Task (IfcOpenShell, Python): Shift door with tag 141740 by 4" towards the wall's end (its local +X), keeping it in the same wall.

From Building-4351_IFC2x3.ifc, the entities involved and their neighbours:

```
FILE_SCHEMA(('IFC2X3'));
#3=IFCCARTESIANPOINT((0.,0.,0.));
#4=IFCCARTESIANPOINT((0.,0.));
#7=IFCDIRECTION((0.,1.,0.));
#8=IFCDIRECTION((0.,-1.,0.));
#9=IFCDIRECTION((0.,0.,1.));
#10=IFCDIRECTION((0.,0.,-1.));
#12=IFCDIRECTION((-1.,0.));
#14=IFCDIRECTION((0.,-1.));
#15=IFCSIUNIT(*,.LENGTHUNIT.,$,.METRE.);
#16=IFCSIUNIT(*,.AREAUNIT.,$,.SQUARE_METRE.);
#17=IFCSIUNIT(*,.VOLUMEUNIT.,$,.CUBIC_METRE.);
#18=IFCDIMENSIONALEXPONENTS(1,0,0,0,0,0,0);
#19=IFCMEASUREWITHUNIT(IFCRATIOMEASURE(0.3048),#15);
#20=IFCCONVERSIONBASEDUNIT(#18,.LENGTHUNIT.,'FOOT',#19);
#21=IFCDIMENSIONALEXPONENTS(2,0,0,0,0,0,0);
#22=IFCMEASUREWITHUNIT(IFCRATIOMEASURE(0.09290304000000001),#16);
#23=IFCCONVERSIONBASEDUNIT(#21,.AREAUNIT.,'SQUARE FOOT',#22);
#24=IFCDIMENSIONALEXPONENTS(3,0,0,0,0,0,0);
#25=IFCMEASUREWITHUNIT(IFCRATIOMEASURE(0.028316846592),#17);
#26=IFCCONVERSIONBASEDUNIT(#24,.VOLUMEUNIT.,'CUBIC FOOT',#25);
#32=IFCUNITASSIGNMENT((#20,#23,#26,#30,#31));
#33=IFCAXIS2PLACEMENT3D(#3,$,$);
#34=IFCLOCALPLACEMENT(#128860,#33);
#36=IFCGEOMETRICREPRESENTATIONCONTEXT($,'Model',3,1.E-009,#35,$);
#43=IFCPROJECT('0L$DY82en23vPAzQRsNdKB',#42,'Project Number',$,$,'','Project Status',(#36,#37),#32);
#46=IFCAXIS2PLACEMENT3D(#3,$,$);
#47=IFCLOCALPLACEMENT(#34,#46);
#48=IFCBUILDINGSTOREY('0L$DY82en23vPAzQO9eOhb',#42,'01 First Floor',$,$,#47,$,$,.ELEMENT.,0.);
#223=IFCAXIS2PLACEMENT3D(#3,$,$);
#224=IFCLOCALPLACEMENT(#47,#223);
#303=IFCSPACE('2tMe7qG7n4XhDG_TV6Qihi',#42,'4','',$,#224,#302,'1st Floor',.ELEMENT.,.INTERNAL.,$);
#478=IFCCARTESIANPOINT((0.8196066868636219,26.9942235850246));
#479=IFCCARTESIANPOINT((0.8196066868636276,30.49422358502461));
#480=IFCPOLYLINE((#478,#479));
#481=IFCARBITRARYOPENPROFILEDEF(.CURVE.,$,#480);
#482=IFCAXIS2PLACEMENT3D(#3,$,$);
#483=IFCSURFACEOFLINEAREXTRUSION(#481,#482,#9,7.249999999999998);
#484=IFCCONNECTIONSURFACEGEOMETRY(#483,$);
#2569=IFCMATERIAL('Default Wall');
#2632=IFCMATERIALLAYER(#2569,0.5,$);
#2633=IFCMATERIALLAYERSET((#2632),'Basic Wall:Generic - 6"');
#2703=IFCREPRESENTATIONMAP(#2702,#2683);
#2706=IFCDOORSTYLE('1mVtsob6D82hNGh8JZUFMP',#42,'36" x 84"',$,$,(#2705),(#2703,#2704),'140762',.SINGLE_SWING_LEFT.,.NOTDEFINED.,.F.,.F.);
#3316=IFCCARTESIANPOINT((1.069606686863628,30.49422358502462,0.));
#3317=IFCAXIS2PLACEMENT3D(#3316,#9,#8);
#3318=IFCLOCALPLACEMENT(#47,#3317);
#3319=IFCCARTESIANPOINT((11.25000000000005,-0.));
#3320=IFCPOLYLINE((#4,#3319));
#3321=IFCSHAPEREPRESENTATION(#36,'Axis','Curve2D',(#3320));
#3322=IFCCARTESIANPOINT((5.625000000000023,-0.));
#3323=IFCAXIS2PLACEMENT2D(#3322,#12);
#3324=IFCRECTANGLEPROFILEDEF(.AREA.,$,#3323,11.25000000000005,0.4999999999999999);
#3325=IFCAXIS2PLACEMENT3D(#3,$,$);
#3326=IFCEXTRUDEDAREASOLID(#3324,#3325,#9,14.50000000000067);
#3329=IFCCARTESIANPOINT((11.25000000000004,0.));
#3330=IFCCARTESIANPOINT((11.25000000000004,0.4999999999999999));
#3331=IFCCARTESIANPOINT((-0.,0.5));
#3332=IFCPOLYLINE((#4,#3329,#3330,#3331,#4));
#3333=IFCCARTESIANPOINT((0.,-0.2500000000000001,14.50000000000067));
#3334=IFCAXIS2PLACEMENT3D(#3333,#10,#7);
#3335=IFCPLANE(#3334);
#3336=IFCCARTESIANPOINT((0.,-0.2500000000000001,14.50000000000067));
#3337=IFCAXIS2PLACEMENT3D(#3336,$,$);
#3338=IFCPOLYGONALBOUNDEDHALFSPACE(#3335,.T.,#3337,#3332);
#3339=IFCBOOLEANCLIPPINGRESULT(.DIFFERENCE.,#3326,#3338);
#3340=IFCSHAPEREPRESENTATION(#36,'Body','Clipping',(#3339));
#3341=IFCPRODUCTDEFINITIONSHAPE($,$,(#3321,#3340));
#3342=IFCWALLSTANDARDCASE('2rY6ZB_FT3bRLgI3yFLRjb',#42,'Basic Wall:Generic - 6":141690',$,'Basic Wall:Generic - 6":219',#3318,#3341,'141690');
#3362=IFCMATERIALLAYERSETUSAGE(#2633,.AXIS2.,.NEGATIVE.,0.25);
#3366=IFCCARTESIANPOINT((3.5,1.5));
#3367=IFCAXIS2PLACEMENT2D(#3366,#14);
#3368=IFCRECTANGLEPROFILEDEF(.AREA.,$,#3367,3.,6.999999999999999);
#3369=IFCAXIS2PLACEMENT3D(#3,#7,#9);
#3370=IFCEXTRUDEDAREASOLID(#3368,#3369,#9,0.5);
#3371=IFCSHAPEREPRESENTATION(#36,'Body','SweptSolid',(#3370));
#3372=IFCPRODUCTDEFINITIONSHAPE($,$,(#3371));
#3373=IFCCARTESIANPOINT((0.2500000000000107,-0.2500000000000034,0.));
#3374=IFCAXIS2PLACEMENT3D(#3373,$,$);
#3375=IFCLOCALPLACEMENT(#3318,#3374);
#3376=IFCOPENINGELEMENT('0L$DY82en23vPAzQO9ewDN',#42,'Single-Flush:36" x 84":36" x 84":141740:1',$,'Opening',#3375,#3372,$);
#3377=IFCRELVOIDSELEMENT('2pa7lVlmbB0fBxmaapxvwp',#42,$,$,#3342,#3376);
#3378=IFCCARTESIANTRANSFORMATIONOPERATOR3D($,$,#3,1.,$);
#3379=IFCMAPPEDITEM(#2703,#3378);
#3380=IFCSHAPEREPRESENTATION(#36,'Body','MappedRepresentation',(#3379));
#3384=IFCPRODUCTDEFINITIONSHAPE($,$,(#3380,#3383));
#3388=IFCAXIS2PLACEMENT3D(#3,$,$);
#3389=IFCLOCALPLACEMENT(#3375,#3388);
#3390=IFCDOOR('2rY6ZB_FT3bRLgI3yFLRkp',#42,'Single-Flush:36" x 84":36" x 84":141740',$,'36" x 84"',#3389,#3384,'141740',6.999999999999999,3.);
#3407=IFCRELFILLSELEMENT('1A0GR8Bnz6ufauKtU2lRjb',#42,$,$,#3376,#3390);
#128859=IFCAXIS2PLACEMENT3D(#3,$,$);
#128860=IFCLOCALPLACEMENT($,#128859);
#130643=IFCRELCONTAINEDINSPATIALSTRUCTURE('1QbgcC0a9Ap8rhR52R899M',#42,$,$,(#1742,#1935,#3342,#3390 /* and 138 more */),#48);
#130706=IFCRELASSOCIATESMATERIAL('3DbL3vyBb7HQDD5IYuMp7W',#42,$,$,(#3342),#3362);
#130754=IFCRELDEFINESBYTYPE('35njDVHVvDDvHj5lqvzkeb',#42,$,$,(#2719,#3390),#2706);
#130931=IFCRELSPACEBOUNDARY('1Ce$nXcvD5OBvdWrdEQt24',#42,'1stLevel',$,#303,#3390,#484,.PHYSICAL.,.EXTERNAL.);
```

```python
import numpy as np
import ifcopenshell
import ifcopenshell.api.geometry
import ifcopenshell.util.placement
import ifcopenshell.util.unit

model = ifcopenshell.open("Building-4351_IFC2x3.ifc")
unit_scale = ifcopenshell.util.unit.calculate_unit_scale(model)

door = model.by_guid("2rY6ZB_FT3bRLgI3yFLRkp")
opening = door.FillsVoids[0].RelatingOpeningElement
wall = opening.VoidsElements[0].RelatingBuildingElement

wall_matrix = ifcopenshell.util.placement.get_local_placement(wall.ObjectPlacement)
shift = wall_matrix[:3, 0] * 4 * 0.0254 / unit_scale
before = ifcopenshell.util.placement.get_local_placement(door.ObjectPlacement)[:3, 3].copy()

# The door is placed relative to its opening, so it follows when the opening moves.
matrix = ifcopenshell.util.placement.get_local_placement(opening.ObjectPlacement)
matrix[:3, 3] += shift
ifcopenshell.api.geometry.edit_object_placement(
    model, product=opening, matrix=matrix, is_si=False, should_transform_children=True
)

# Space boundary surfaces are stored in each space's coordinates; move them too.
for rel in door.ProvidesBoundaries:
    if not rel.ConnectionGeometry:
        continue
    surface = rel.ConnectionGeometry.SurfaceOnRelatingElement
    space_matrix = ifcopenshell.util.placement.get_local_placement(rel.RelatingSpace.ObjectPlacement)
    point = np.array(surface.Position.Location.Coordinates) + space_matrix[:3, :3].T @ shift
    surface.Position = model.createIfcAxis2Placement3D(
        model.createIfcCartesianPoint(point.tolist()), surface.Position.Axis, surface.Position.RefDirection
    )

after = ifcopenshell.util.placement.get_local_placement(door.ObjectPlacement)[:3, 3]
print("door moved by", (after - before).round(3) + 0.0)

model.write("Building-4351_IFC2x3_rev.ifc")
```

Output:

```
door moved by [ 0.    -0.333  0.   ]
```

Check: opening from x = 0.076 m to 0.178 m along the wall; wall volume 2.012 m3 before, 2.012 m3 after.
